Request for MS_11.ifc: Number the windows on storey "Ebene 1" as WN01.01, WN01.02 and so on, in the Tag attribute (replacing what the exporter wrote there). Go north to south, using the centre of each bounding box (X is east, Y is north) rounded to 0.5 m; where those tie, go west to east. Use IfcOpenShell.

First a look at what the model holds.

```python
import ifcopenshell
import ifcopenshell.util.element
import ifcopenshell.util.placement

model = ifcopenshell.open("MS_11.ifc")
print(model.schema)
storey = next(s for s in model.by_type("IfcBuildingStorey") if s.Name == "Ebene 1")
windows = [e for e in ifcopenshell.util.element.get_decomposition(storey) if e.is_a("IfcWindow")]
for e in sorted(windows, key=lambda e: e.id()):
    origin = ifcopenshell.util.placement.get_local_placement(e.ObjectPlacement)[:3, 3]
    print(e.id(), e.Tag, e.Name, origin.round(2) + 0.0, sep=" | ")
```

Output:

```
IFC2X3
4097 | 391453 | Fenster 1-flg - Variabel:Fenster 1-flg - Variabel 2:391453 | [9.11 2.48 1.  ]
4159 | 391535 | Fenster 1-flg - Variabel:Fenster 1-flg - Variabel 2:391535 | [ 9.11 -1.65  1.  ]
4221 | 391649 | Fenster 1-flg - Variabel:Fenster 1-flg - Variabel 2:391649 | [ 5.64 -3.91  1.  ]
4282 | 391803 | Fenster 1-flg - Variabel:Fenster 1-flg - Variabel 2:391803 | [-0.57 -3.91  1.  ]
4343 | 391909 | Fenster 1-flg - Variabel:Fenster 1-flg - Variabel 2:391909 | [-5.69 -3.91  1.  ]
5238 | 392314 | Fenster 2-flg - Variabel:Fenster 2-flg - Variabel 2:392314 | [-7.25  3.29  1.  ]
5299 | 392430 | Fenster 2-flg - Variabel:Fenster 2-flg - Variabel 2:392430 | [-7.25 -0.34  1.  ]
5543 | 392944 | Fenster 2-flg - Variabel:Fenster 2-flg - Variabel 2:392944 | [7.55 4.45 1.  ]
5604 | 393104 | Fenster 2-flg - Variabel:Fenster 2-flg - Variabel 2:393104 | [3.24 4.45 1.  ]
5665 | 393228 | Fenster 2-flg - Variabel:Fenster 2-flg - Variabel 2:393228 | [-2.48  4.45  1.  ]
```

```python
import ifcopenshell
import ifcopenshell.geom
import ifcopenshell.util.element
import ifcopenshell.util.shape

model = ifcopenshell.open("MS_11.ifc")
settings = ifcopenshell.geom.settings()
settings.set("use-world-coords", True)


def centre(element):
    shape = ifcopenshell.geom.create_shape(settings, element)
    return ifcopenshell.util.shape.get_bbox_centroid(shape.geometry)


storey = next(s for s in model.by_type("IfcBuildingStorey") if s.Name == "Ebene 1")
windows = [e for e in ifcopenshell.util.element.get_decomposition(storey) if e.is_a("IfcWindow")]

# Insertion points can sit at a corner or the storey origin, so sort by the geometry (in metres).
centres = {e: centre(e) for e in windows}
windows.sort(key=lambda e: (-round(centres[e][1] / 0.5), centres[e][0]))

for i, e in enumerate(windows, start=1):
    number = f"WN01.{i:02d}"
    e.Tag = number
    print(e.id(), number)

model.write("MS_11_rev.ifc")
```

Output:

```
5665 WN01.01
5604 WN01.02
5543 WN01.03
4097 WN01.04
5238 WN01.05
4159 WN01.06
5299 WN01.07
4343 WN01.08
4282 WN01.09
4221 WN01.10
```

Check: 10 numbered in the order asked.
